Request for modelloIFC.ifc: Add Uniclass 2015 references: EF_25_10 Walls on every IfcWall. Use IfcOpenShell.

First a look at what the model holds.

```python
import ifcopenshell

model = ifcopenshell.open("modelloIFC.ifc")
print(model.schema)
print("classifications:", [c.Name for c in model.by_type("IfcClassification")])
for ifc_class in ("IfcDoor", "IfcRoof", "IfcStair", "IfcWall", "IfcWindow"):
    print(ifc_class, len(model.by_type(ifc_class)))
```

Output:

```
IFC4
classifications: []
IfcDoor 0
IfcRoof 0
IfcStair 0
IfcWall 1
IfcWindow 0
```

```python
import ifcopenshell
import ifcopenshell.api.classification

model = ifcopenshell.open("modelloIFC.ifc")

system = ifcopenshell.api.classification.add_classification(model, classification="Uniclass 2015")

codes = {
    "IfcWall": ("EF_25_10", "Walls"),
}
for ifc_class, (code, name) in codes.items():
    products = model.by_type(ifc_class)
    ifcopenshell.api.classification.add_reference(
        model, products=products, classification=system, identification=code, name=name
    )
    print(code, len(products))

model.write("modelloIFC-out.ifc")
```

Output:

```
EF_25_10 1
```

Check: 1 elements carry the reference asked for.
